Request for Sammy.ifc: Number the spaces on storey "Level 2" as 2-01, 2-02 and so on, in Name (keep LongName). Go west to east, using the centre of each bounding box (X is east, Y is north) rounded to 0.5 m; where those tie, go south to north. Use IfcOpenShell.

First a look at what the model holds.

```python
import ifcopenshell
import ifcopenshell.util.element
import ifcopenshell.util.placement

model = ifcopenshell.open("Sammy.ifc")
print(model.schema)
storey = next(s for s in model.by_type("IfcBuildingStorey") if s.Name == "Level 2")
spaces = [e for e in ifcopenshell.util.element.get_decomposition(storey) if e.is_a("IfcSpace")]
for e in sorted(spaces, key=lambda e: e.id()):
    origin = ifcopenshell.util.placement.get_local_placement(e.ObjectPlacement)[:3, 3]
    print(e.id(), e.Name, e.LongName, origin.round(2) + 0.0, sep=" | ")
```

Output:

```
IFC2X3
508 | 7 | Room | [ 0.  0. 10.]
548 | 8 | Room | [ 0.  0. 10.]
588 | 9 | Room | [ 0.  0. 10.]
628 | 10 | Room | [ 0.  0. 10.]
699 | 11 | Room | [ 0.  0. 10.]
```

```python
import ifcopenshell
import ifcopenshell.geom
import ifcopenshell.util.element
import ifcopenshell.util.shape

model = ifcopenshell.open("Sammy.ifc")
settings = ifcopenshell.geom.settings()
settings.set("use-world-coords", True)


def centre(element):
    shape = ifcopenshell.geom.create_shape(settings, element)
    return ifcopenshell.util.shape.get_bbox_centroid(shape.geometry)


storey = next(s for s in model.by_type("IfcBuildingStorey") if s.Name == "Level 2")
spaces = [e for e in ifcopenshell.util.element.get_decomposition(storey) if e.is_a("IfcSpace")]

# Insertion points can sit at a corner or the storey origin, so sort by the geometry (in metres).
centres = {e: centre(e) for e in spaces}
spaces.sort(key=lambda e: (round(centres[e][0] / 0.5), centres[e][1]))

for i, e in enumerate(spaces, start=1):
    number = f"2-{i:02d}"
    e.Name = number
    print(e.id(), number)

model.write("Sammy_updated.ifc")
```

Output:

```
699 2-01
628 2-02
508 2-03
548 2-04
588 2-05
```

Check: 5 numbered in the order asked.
